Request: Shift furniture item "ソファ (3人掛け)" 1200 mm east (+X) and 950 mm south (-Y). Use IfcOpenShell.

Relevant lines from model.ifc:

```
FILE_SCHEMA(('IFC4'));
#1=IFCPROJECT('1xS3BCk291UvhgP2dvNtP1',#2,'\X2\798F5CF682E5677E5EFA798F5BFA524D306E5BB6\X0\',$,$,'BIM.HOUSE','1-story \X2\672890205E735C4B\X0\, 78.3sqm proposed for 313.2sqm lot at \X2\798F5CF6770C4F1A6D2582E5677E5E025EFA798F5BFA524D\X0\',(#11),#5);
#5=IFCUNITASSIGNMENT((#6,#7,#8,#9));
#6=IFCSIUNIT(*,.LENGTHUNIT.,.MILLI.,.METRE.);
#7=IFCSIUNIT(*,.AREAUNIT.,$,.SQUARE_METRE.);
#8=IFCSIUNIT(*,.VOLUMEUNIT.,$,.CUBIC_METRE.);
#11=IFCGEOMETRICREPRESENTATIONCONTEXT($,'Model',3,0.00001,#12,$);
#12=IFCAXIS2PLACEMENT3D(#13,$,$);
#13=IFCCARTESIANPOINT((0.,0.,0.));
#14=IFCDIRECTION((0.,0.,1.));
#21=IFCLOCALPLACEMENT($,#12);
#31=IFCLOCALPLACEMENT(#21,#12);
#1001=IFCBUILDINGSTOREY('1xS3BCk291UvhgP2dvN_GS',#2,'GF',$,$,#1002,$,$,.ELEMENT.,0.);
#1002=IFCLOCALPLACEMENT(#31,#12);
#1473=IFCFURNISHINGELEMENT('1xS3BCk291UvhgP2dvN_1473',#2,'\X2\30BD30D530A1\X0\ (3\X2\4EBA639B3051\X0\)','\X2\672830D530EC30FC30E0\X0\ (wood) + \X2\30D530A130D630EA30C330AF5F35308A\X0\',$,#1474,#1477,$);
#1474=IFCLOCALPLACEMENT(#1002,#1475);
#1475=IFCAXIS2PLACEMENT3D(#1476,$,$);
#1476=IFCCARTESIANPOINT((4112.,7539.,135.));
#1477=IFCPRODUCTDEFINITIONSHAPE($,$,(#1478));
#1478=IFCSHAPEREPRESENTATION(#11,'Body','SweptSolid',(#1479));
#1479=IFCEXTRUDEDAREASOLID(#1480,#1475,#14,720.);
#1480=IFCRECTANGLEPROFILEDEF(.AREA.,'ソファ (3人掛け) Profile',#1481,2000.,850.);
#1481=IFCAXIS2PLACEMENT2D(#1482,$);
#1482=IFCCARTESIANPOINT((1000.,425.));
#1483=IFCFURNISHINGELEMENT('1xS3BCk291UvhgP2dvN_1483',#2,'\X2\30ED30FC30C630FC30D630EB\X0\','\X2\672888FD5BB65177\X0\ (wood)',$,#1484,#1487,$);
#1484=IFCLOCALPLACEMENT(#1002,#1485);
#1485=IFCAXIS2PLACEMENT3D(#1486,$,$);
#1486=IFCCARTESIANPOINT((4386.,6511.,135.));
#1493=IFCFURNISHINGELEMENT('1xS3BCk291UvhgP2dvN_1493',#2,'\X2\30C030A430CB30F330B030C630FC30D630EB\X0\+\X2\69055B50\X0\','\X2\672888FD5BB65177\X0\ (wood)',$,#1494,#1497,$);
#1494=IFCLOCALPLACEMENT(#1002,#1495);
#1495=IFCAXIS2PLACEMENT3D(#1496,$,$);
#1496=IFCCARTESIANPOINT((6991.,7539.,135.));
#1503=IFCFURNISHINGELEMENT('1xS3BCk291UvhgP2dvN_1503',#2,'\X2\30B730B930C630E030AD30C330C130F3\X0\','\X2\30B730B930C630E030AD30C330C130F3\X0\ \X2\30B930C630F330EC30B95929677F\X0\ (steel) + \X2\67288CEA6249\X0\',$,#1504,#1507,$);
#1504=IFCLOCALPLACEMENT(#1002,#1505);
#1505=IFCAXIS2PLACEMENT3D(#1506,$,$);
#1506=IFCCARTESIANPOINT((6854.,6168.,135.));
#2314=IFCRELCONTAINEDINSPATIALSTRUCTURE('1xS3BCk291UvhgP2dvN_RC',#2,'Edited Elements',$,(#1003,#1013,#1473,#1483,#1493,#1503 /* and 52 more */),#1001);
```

```python
import ifcopenshell
import ifcopenshell.api.geometry
import ifcopenshell.util.placement
import ifcopenshell.util.unit

model = ifcopenshell.open("model.ifc")
unit_scale = ifcopenshell.util.unit.calculate_unit_scale(model)

item = model.by_id(1473)
matrix = ifcopenshell.util.placement.get_local_placement(item.ObjectPlacement)
matrix[0, 3] += 1.2 / unit_scale
matrix[1, 3] -= 0.95 / unit_scale
ifcopenshell.api.geometry.edit_object_placement(model, product=item, matrix=matrix, is_si=False)

print(ifcopenshell.util.placement.get_local_placement(item.ObjectPlacement).round(3) + 0.0)

model.write("model-out.ifc")
```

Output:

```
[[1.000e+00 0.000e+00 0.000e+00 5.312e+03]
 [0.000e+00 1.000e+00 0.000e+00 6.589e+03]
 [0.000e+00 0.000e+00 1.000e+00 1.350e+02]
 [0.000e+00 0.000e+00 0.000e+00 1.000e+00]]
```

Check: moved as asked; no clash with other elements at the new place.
